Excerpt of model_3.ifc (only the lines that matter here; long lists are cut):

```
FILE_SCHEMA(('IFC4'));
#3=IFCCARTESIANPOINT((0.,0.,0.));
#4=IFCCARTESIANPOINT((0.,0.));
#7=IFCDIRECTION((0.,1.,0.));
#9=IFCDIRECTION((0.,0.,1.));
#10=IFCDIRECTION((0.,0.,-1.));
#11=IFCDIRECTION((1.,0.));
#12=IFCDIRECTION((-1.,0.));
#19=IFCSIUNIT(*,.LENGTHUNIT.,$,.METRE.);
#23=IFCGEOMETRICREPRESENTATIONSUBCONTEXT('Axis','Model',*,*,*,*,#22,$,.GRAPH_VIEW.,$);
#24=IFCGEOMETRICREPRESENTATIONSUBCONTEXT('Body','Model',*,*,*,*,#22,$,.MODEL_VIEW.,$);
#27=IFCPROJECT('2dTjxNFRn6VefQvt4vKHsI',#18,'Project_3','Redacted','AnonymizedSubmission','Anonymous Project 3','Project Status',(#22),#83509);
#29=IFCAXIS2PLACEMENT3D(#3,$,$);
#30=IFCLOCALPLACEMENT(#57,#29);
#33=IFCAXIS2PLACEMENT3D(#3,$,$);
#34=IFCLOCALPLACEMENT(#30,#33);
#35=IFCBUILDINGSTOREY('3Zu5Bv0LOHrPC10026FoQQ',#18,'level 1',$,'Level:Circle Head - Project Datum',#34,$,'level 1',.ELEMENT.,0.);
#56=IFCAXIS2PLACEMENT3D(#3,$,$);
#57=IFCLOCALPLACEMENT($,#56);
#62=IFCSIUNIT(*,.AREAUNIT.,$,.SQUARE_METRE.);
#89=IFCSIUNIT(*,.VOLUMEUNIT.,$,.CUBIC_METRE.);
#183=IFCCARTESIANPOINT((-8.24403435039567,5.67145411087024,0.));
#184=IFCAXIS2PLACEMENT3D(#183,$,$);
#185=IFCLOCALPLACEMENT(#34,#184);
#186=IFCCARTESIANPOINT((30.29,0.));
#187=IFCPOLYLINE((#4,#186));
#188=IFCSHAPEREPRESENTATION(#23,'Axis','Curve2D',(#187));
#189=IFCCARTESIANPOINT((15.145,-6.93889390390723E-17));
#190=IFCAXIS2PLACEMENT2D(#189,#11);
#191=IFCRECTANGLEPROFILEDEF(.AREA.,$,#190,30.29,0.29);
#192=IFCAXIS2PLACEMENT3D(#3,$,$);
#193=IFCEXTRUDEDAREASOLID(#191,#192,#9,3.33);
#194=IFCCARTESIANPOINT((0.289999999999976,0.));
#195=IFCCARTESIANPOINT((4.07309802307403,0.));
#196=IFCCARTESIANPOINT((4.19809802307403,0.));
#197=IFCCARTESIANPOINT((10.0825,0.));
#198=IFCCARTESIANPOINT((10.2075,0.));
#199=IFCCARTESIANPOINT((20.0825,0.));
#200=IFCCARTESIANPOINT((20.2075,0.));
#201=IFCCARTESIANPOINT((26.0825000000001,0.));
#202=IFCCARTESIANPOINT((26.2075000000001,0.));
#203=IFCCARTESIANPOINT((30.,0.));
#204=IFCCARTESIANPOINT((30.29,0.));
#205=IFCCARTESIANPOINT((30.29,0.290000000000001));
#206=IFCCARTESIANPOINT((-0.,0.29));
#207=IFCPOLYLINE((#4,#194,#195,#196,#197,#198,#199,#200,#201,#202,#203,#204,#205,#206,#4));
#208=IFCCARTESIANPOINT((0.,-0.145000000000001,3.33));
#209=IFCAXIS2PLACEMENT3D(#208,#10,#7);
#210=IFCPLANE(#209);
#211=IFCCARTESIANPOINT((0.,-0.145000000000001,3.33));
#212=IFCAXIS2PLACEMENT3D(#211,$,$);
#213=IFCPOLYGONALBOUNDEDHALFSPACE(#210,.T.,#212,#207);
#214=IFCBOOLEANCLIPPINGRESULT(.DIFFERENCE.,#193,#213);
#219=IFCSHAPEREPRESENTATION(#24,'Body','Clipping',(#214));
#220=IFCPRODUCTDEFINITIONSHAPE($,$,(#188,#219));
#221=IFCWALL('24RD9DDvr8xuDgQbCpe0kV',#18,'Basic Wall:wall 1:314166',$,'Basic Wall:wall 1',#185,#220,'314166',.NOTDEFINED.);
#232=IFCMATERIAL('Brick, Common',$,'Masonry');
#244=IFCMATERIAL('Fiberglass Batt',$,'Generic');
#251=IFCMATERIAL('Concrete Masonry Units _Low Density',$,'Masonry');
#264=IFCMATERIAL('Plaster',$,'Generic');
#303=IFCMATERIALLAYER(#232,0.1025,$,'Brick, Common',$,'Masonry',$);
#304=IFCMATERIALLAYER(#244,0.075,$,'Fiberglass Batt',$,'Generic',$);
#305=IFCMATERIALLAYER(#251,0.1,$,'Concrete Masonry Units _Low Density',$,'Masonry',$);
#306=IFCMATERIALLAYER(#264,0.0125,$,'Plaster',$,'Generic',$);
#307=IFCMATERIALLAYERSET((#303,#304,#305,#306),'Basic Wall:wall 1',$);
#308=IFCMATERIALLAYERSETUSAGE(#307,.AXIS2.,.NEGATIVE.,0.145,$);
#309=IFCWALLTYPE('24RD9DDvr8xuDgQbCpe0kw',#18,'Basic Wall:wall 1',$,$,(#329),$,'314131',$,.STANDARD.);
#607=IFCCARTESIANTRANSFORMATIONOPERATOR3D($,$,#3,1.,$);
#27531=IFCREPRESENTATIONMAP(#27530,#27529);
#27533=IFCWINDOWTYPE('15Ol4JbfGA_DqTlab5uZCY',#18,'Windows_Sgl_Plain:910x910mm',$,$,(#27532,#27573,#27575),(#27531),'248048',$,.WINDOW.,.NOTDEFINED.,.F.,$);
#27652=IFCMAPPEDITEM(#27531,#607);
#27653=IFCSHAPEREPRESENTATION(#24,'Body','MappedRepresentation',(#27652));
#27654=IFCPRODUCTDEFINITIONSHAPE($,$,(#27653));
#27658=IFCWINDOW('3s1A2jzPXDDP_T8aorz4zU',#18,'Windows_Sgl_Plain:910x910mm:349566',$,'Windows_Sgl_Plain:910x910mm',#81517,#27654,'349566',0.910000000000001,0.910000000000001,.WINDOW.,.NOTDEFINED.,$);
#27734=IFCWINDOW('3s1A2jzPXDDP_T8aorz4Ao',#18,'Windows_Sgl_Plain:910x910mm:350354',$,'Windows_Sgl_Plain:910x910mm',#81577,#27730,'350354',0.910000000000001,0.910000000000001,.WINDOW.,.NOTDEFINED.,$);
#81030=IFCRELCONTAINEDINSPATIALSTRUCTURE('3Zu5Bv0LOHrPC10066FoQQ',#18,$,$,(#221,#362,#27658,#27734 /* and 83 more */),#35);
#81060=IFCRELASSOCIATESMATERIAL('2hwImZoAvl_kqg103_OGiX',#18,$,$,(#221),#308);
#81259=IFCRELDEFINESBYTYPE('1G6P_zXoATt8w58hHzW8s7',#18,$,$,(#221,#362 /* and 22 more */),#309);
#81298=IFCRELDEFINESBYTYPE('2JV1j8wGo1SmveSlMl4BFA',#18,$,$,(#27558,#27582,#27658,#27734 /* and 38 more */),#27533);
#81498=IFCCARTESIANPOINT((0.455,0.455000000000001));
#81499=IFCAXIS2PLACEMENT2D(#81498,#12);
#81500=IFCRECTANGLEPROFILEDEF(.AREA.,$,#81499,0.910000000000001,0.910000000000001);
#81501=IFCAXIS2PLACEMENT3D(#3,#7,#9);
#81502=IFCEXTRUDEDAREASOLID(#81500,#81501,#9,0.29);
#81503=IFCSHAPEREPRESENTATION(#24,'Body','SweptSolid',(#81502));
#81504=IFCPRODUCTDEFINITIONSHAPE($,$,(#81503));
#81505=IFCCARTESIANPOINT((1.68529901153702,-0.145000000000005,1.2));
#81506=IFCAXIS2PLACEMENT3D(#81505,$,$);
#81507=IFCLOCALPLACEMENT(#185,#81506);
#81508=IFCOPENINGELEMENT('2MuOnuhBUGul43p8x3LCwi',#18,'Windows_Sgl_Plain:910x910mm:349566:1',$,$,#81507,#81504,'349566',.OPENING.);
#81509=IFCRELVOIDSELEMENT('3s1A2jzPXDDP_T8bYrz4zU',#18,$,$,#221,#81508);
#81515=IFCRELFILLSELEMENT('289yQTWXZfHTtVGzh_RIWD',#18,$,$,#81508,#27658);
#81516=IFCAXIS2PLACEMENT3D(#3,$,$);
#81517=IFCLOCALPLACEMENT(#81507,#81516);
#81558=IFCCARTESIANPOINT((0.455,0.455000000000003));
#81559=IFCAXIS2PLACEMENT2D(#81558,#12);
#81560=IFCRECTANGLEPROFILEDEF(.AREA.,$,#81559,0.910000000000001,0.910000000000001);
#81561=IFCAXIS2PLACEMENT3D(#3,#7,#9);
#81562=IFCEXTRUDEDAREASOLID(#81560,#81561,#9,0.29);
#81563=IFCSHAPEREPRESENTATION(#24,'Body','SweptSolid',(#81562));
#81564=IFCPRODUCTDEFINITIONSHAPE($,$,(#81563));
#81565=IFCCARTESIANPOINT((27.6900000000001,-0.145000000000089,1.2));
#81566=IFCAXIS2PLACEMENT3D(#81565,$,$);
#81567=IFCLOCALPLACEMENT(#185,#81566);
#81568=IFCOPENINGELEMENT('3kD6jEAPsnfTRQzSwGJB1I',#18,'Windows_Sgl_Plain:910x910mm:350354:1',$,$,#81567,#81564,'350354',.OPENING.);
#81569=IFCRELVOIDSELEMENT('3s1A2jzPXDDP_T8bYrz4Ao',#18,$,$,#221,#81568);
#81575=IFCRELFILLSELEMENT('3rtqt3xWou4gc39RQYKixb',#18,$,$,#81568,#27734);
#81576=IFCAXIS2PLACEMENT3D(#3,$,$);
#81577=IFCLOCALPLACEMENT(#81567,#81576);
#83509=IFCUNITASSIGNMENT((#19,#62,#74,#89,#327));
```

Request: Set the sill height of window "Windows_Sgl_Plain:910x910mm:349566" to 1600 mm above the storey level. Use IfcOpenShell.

```python
import numpy as np
import ifcopenshell
import ifcopenshell.api.geometry
import ifcopenshell.geom
import ifcopenshell.util.element
import ifcopenshell.util.placement
import ifcopenshell.util.shape
import ifcopenshell.util.unit

model = ifcopenshell.open("model_3.ifc")
unit_scale = ifcopenshell.util.unit.calculate_unit_scale(model)

window = model.by_guid("3s1A2jzPXDDP_T8aorz4zU")
opening = window.FillsVoids[0].RelatingOpeningElement
storey = ifcopenshell.util.element.get_container(window, ifc_class="IfcBuildingStorey")
level = ifcopenshell.util.placement.get_local_placement(storey.ObjectPlacement)[2, 3]

# The opening's origin need not be at the sill, so measure its lowest point.
shape = ifcopenshell.geom.create_shape(ifcopenshell.geom.settings(), opening)
bottom = ifcopenshell.util.shape.get_shape_bottom_elevation(shape, shape.geometry) / unit_scale
dz = level + 1.6 / unit_scale - bottom

shift = np.array([0.0, 0.0, dz])
# The window is placed relative to its opening, so it follows when the opening moves.
matrix = ifcopenshell.util.placement.get_local_placement(opening.ObjectPlacement)
matrix[:3, 3] += shift
ifcopenshell.api.geometry.edit_object_placement(
    model, product=opening, matrix=matrix, is_si=False, should_transform_children=True
)

print(f"moved by {dz * unit_scale:+.3f} m")

model.write("model_3_updated.ifc")
```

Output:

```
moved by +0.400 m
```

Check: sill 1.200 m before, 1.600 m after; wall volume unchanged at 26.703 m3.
